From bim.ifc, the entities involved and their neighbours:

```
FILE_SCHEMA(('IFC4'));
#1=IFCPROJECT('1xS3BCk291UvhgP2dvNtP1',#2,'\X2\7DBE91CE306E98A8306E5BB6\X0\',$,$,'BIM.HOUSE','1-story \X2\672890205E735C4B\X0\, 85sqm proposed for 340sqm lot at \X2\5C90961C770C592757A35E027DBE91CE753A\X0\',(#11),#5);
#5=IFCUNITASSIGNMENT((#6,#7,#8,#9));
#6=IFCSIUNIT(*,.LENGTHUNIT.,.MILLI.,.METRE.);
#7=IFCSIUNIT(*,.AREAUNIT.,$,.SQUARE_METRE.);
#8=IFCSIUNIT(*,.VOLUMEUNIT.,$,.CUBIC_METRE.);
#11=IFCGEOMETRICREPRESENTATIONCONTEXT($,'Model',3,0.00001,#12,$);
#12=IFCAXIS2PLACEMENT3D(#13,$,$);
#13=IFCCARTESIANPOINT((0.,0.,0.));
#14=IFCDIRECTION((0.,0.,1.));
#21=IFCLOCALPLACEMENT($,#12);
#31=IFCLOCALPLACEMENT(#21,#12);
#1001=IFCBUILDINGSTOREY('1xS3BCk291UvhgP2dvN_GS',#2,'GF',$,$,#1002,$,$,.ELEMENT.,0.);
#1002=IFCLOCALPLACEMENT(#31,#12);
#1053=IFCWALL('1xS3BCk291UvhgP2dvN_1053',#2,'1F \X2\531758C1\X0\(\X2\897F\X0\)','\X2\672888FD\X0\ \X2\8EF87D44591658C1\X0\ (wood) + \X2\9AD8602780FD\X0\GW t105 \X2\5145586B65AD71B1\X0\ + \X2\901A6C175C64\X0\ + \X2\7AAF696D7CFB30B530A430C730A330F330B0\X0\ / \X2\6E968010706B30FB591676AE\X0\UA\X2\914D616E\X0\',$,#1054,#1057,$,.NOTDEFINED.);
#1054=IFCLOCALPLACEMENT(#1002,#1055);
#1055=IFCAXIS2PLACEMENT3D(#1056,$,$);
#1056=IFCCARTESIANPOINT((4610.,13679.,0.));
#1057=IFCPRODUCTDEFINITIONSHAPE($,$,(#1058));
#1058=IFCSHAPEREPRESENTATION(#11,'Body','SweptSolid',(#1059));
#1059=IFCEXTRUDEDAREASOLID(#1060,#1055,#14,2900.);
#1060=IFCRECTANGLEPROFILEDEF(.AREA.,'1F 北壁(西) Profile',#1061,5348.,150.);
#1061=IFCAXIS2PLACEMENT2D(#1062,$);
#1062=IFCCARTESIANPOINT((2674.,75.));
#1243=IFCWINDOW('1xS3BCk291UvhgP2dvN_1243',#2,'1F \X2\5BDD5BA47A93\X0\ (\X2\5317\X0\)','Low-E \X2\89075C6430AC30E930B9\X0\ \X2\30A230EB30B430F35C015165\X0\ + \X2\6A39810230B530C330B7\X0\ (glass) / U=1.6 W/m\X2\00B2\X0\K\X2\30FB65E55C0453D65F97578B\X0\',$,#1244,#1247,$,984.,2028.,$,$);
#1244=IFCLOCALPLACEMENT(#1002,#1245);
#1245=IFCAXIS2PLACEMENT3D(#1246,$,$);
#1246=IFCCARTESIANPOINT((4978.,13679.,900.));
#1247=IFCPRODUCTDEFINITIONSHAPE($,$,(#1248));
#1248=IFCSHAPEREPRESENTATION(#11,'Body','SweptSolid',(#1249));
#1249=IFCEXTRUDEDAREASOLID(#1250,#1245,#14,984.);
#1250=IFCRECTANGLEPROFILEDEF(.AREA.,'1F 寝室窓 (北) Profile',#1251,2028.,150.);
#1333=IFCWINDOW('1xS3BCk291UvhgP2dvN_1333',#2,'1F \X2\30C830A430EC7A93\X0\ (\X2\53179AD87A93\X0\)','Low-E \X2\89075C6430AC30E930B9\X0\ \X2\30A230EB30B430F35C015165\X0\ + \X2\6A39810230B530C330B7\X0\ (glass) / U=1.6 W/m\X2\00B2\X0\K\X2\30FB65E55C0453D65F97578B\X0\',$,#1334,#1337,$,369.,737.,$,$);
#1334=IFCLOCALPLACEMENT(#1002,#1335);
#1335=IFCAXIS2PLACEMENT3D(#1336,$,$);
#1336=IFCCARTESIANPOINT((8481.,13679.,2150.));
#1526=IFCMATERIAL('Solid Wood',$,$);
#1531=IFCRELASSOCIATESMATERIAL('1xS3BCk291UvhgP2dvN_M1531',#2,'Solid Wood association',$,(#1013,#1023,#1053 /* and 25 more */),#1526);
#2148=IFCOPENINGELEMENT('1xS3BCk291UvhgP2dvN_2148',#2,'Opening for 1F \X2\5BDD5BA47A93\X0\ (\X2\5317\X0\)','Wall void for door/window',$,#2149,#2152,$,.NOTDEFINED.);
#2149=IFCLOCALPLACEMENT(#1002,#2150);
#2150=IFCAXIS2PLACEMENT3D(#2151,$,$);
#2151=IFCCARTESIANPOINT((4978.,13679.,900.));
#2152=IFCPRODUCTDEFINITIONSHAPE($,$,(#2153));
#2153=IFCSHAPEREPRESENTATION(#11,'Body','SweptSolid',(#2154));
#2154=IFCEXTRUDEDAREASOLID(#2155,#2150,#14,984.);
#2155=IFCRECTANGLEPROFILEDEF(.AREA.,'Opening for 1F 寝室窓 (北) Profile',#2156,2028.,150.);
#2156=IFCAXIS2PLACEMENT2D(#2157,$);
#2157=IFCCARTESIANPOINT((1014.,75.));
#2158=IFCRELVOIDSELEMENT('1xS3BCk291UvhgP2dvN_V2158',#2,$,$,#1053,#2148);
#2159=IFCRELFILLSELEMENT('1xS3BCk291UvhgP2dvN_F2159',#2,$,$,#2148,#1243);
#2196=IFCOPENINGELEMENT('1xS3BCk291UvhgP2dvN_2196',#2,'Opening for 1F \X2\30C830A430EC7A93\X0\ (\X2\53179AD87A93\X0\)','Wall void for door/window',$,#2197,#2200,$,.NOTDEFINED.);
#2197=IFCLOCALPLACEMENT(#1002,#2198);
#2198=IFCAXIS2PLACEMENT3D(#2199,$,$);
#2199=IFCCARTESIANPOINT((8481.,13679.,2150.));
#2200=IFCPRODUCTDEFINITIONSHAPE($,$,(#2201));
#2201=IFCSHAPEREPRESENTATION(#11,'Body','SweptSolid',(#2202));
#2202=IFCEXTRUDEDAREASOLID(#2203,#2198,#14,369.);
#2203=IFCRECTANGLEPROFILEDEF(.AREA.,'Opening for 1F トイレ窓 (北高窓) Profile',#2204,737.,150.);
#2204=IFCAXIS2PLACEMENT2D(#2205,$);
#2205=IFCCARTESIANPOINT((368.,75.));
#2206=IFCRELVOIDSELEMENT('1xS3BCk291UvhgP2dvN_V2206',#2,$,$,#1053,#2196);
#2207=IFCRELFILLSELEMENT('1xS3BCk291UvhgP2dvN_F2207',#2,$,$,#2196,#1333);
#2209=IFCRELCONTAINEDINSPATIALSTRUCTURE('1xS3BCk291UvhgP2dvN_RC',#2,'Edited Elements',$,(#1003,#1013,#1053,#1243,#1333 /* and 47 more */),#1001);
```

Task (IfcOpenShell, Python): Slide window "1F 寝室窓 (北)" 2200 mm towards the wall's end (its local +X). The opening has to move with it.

```python
import ifcopenshell
import ifcopenshell.api.geometry
import ifcopenshell.util.placement

model = ifcopenshell.open("bim.ifc")

window = model.by_guid("1xS3BCk291UvhgP2dvN_1243")
opening = window.FillsVoids[0].RelatingOpeningElement
wall = opening.VoidsElements[0].RelatingBuildingElement

wall_matrix = ifcopenshell.util.placement.get_local_placement(wall.ObjectPlacement)
shift = wall_matrix[:3, 0] * 2200.0
before = ifcopenshell.util.placement.get_local_placement(window.ObjectPlacement)[:3, 3].copy()

# The window is not placed relative to its opening, so move both.
for product in (opening, window):
    matrix = ifcopenshell.util.placement.get_local_placement(product.ObjectPlacement)
    matrix[:3, 3] += shift
    ifcopenshell.api.geometry.edit_object_placement(model, product=product, matrix=matrix, is_si=False)

after = ifcopenshell.util.placement.get_local_placement(window.ObjectPlacement)[:3, 3]
print("window moved by", (after - before).round(3) + 0.0)

model.write("bim_edited.ifc")
```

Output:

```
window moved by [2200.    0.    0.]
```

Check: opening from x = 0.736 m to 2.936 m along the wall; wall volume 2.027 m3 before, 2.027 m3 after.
